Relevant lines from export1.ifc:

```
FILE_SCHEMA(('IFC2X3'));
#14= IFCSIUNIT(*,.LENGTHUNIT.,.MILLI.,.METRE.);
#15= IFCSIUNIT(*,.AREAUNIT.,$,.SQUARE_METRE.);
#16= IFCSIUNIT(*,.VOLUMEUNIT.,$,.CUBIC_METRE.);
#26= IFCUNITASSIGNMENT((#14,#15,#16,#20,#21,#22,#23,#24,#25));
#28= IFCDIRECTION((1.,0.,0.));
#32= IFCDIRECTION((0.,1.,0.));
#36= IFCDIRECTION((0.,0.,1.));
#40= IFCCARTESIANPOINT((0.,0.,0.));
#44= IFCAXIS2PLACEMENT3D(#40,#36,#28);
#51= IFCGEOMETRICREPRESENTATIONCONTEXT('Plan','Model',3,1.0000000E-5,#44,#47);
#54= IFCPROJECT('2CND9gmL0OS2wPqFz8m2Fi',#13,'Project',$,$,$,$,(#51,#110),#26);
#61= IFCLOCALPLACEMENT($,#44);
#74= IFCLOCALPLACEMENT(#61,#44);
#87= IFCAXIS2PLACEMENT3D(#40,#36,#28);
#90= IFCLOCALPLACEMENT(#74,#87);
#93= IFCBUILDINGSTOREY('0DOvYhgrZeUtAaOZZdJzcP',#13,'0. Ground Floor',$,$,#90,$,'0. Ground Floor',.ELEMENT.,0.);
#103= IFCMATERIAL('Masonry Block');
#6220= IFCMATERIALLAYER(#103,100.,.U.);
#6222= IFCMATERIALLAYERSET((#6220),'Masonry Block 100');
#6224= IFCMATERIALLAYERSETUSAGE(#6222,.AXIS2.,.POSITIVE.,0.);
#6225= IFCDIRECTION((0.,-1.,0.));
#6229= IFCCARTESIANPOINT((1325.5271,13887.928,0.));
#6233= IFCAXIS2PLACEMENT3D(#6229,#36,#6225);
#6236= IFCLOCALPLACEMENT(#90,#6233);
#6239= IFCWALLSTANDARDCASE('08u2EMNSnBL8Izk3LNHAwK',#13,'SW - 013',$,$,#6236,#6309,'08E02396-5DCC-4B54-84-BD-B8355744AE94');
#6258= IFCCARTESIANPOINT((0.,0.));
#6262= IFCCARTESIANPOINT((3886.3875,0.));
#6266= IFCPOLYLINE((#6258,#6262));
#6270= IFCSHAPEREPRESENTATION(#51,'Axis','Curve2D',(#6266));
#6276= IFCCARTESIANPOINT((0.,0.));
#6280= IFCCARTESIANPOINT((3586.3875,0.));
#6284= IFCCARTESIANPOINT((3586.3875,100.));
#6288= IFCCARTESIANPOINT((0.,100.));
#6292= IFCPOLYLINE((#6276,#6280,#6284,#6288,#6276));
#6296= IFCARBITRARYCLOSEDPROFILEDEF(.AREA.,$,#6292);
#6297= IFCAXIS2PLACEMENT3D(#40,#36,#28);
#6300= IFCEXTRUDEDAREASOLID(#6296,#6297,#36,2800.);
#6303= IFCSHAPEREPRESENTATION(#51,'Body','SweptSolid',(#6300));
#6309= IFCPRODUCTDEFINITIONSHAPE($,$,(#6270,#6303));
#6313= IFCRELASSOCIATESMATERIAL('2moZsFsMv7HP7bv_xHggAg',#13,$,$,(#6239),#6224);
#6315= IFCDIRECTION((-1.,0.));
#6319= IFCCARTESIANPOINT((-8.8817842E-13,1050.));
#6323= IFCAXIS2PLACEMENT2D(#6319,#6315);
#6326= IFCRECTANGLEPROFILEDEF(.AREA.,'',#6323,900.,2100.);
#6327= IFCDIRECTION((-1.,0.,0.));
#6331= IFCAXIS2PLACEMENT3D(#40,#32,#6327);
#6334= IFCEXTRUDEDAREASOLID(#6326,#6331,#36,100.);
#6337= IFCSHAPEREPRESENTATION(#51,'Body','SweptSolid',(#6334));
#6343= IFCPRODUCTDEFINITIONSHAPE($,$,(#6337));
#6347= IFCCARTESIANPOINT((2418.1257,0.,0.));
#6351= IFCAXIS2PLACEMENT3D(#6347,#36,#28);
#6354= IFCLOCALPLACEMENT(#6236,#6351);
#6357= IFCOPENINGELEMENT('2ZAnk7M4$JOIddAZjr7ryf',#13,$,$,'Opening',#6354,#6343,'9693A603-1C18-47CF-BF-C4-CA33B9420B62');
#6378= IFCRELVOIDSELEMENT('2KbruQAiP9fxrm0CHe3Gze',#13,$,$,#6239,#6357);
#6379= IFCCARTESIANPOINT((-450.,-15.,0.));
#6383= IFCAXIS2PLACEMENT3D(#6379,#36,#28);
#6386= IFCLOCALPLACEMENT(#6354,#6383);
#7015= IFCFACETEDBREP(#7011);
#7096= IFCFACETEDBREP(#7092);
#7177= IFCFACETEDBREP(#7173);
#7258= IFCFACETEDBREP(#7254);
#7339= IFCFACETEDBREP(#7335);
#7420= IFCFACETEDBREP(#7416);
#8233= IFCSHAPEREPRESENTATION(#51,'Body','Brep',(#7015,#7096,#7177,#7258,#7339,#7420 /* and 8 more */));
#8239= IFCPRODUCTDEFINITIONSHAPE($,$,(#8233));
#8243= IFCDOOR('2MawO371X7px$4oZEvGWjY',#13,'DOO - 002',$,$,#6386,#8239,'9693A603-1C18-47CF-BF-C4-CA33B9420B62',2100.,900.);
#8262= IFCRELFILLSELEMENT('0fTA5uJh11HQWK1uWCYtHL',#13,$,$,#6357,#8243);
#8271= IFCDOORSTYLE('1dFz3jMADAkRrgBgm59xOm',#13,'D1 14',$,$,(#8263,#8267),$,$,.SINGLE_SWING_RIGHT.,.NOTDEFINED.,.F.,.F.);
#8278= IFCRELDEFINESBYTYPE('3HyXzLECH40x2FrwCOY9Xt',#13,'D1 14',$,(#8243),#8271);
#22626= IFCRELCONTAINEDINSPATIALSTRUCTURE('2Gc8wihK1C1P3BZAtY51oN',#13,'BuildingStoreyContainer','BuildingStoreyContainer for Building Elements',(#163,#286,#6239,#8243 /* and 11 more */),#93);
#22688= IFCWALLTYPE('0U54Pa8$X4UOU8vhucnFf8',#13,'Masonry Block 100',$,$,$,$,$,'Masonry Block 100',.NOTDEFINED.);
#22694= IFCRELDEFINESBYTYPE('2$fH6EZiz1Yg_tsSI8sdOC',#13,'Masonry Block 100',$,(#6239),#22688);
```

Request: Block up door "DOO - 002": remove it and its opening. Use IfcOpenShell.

```python
import ifcopenshell
import ifcopenshell.api.feature
import ifcopenshell.api.root
import ifcopenshell.geom
import ifcopenshell.util.shape

model = ifcopenshell.open("export1.ifc")
settings = ifcopenshell.geom.settings()


def volume(element):
    """Net volume in cubic metres, openings subtracted."""
    shape = ifcopenshell.geom.create_shape(settings, element)
    return ifcopenshell.util.shape.get_volume(shape.geometry)


door = model.by_id(8243)
opening = door.FillsVoids[0].RelatingOpeningElement
wall = opening.VoidsElements[0].RelatingBuildingElement
before = volume(wall)

ifcopenshell.api.root.remove_product(model, product=door)
ifcopenshell.api.feature.remove_feature(model, feature=opening)

after = volume(wall)

print(f"wall volume {before:.3f} -> {after:.3f} m3")

model.write("export1_rev.ifc")
```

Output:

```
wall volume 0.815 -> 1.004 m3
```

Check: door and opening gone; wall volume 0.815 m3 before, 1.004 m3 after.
